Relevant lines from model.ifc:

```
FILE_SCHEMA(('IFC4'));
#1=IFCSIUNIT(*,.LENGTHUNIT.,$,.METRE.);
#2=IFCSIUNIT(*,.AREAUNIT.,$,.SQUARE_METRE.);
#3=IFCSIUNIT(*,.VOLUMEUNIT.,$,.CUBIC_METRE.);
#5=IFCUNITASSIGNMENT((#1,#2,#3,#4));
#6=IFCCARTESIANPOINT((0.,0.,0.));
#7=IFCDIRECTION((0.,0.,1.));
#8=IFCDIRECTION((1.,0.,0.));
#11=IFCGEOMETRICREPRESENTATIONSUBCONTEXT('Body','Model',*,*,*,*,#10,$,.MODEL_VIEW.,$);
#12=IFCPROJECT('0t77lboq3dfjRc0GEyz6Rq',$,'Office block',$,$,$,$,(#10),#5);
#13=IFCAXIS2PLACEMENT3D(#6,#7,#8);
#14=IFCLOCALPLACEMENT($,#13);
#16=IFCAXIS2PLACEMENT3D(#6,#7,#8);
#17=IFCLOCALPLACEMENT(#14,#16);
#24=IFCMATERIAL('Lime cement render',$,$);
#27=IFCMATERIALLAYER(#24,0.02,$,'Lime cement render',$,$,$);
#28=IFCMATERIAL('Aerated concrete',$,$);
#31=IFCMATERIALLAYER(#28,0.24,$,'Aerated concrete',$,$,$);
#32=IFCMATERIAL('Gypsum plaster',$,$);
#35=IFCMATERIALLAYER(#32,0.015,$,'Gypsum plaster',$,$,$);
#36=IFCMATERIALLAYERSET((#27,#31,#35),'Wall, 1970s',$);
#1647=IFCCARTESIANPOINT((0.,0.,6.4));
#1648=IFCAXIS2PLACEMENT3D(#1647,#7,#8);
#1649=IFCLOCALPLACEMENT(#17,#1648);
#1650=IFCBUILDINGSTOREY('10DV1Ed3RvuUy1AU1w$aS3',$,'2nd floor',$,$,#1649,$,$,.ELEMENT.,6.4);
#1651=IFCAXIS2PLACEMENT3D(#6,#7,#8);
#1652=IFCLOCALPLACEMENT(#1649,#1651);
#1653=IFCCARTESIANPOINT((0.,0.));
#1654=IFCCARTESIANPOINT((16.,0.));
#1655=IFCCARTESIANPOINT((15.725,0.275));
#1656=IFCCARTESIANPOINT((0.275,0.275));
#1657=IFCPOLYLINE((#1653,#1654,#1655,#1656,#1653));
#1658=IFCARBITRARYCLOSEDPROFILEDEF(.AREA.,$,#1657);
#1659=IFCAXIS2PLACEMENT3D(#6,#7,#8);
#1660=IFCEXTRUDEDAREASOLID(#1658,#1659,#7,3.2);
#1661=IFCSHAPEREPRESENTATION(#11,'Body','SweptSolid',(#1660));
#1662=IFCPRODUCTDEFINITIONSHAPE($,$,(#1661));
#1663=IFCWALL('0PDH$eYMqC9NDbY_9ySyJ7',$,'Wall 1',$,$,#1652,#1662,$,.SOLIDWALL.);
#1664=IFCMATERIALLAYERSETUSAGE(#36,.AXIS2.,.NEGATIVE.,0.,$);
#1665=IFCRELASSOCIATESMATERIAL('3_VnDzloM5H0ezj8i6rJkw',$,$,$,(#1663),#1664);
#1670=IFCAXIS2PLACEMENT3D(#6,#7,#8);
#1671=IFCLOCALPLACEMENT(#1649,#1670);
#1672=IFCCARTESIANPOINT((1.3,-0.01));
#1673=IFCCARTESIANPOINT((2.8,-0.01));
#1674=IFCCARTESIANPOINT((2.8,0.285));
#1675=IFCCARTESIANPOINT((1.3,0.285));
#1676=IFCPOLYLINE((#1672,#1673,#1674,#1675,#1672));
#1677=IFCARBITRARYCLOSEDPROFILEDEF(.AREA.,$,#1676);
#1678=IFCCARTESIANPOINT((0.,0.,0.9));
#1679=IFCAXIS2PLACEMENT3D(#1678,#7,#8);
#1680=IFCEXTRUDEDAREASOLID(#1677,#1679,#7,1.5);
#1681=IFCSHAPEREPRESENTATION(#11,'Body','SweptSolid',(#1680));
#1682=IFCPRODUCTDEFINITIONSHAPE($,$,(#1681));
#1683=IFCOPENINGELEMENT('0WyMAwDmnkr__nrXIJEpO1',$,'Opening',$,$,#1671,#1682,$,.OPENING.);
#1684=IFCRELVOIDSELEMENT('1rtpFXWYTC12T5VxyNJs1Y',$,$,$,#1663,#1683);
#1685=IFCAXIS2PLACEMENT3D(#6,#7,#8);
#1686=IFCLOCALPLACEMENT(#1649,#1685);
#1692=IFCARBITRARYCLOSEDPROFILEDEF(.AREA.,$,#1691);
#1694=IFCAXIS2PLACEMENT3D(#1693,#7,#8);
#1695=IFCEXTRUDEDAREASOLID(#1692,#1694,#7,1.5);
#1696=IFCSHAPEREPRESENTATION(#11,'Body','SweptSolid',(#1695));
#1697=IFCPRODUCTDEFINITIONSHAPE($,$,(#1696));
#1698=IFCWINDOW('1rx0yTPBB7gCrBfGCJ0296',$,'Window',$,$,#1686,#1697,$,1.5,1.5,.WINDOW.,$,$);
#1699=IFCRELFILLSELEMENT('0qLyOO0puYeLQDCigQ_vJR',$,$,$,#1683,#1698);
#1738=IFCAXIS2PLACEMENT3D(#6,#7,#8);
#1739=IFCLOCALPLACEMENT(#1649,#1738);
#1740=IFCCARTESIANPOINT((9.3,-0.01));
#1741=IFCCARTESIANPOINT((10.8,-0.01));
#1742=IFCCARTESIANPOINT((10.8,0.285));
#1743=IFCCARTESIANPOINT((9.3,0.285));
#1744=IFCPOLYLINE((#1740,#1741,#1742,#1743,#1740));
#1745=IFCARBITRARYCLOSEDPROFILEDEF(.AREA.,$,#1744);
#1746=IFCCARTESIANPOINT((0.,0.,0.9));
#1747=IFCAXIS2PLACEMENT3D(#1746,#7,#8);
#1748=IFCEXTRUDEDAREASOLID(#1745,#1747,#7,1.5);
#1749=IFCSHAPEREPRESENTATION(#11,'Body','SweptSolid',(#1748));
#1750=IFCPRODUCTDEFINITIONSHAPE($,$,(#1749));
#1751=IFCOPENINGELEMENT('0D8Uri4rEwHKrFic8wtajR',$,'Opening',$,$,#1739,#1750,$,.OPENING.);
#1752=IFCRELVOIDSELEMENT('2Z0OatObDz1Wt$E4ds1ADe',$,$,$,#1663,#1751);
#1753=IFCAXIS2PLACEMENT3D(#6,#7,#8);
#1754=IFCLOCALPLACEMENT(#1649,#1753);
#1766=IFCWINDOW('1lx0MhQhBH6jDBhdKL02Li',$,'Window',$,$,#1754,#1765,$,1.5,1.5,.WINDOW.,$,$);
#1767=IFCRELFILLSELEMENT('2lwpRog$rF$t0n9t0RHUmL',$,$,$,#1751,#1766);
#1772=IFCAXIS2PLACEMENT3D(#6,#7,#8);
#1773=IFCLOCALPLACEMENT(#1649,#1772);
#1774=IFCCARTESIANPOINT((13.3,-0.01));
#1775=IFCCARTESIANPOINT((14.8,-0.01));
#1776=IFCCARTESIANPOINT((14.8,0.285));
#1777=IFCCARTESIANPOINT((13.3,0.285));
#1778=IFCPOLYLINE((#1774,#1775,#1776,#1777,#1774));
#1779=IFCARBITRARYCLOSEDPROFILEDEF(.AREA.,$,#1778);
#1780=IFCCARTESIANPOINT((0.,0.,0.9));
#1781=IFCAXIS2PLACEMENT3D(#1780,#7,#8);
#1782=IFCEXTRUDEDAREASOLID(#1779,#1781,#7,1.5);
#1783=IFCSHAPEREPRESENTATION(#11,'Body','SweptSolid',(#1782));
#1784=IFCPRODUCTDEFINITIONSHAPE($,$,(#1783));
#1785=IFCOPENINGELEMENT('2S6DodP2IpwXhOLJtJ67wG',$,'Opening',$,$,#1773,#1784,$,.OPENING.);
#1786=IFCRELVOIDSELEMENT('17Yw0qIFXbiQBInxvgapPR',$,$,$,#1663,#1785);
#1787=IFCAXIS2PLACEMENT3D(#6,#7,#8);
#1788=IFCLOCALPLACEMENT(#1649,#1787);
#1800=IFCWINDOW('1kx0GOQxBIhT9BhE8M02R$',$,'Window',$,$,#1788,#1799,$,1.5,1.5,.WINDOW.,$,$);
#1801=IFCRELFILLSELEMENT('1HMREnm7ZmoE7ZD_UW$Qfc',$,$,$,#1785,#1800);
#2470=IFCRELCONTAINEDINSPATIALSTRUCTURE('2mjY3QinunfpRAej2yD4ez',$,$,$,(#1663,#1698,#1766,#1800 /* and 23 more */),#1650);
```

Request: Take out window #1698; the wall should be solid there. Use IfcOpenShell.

```python
import ifcopenshell
import ifcopenshell.api.feature
import ifcopenshell.api.root
import ifcopenshell.geom
import ifcopenshell.util.shape

model = ifcopenshell.open("model.ifc")
settings = ifcopenshell.geom.settings()


def volume(element):
    """Net volume in cubic metres, openings subtracted."""
    shape = ifcopenshell.geom.create_shape(settings, element)
    return ifcopenshell.util.shape.get_volume(shape.geometry)


window = model.by_guid("1rx0yTPBB7gCrBfGCJ0296")
opening = window.FillsVoids[0].RelatingOpeningElement
wall = opening.VoidsElements[0].RelatingBuildingElement
before = volume(wall)

ifcopenshell.api.root.remove_product(model, product=window)
ifcopenshell.api.feature.remove_feature(model, feature=opening)

after = volume(wall)

print(f"wall volume {before:.3f} -> {after:.3f} m3")

model.write("model_edited.ifc")
```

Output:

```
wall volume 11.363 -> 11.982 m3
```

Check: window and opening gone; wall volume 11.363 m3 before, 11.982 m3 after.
